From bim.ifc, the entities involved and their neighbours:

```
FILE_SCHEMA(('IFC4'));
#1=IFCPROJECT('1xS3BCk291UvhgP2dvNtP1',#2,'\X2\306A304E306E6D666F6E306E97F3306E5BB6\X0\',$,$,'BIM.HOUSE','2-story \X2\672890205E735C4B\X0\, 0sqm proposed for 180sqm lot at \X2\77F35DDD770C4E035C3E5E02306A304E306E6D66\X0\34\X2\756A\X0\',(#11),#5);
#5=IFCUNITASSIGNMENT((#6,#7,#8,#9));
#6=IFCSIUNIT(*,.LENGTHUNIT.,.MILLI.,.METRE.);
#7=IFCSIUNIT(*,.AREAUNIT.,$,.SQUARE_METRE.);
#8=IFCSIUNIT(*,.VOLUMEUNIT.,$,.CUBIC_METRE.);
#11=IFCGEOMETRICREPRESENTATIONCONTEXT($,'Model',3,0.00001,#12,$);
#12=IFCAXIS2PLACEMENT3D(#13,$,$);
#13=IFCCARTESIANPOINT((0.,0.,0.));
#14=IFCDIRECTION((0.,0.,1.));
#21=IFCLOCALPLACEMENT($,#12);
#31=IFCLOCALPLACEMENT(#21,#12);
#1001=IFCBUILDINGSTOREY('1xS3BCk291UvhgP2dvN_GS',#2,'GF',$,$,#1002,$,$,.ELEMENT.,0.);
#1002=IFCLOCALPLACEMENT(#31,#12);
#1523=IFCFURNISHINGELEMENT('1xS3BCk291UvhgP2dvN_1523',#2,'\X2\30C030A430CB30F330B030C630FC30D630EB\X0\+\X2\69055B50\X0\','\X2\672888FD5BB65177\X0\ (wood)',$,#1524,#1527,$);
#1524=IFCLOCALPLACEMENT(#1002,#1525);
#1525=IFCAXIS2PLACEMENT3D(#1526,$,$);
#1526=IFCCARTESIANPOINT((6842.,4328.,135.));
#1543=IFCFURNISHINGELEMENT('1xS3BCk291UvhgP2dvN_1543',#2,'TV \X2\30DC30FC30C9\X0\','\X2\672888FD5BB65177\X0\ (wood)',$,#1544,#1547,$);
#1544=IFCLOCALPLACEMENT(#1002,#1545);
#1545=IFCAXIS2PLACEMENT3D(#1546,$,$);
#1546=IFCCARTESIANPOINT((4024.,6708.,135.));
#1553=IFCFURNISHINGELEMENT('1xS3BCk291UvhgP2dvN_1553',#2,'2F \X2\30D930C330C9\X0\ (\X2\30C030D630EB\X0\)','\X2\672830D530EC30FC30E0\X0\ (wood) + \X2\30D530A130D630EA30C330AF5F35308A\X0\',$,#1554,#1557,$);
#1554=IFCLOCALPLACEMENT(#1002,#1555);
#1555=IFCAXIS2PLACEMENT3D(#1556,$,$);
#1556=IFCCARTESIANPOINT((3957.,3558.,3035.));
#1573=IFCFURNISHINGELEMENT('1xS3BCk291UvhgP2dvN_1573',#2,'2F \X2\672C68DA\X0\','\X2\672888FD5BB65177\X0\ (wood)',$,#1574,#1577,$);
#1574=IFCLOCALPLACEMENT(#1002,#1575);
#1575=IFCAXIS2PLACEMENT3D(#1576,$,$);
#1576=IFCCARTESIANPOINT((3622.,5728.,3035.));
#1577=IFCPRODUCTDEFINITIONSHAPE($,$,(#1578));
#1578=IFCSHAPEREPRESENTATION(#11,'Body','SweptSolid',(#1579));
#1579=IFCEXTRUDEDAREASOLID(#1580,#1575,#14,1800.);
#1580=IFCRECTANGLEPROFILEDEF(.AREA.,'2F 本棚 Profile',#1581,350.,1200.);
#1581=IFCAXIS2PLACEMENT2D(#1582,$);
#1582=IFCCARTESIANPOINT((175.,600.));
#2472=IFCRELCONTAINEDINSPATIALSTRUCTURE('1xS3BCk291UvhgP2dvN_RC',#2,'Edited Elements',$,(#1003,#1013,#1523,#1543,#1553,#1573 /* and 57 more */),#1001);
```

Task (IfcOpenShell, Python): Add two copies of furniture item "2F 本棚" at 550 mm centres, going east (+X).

```python
import numpy as np
import ifcopenshell
import ifcopenshell.api.geometry
import ifcopenshell.api.root
import ifcopenshell.util.element
import ifcopenshell.util.placement
import ifcopenshell.util.unit

model = ifcopenshell.open("bim.ifc")
unit_scale = ifcopenshell.util.unit.calculate_unit_scale(model)


def reuse_history(source, copy):
    """copy_class also copies each property set's owner history, people and application; keep the originals."""
    for rel in copy.IsDefinedBy:
        if rel.is_a("IfcRelDefinesByProperties") and (history := rel.RelatingPropertyDefinition.OwnerHistory):
            rel.RelatingPropertyDefinition.OwnerHistory = source.OwnerHistory
            ifcopenshell.util.element.remove_deep2(model, history)


source = model.by_guid("1xS3BCk291UvhgP2dvN_1573")
base = ifcopenshell.util.placement.get_local_placement(source.ObjectPlacement)
step = np.array([1.0, 0.0, 0.0]) * 0.55 / unit_scale

for i in range(1, 3):
    copy = ifcopenshell.api.root.copy_class(model, product=source)
    copy.Representation = ifcopenshell.util.element.copy_deep(
        model, source.Representation, exclude=["IfcGeometricRepresentationContext", "IfcRepresentationMap"]
    )
    reuse_history(source, copy)
    matrix = base.copy()
    matrix[:3, 3] += i * step
    print("added at", matrix[:3, 3].round(3) + 0.0)
    ifcopenshell.api.geometry.edit_object_placement(model, product=copy, matrix=matrix, is_si=False)

model.write("bim_updated.ifc")
```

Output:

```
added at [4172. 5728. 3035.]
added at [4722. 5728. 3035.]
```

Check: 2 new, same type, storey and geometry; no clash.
